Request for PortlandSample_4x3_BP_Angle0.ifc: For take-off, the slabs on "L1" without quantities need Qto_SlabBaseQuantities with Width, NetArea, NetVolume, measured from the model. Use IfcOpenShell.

First a look at what the model holds.

```python
import ifcopenshell
import ifcopenshell.util.element
import ifcopenshell.util.unit

model = ifcopenshell.open("PortlandSample_4x3_BP_Angle0.ifc")
print(model.schema)
for unit_type in ("LENGTHUNIT", "AREAUNIT", "VOLUMEUNIT"):
    print(unit_type, ifcopenshell.util.unit.calculate_unit_scale(model, unit_type))
storey = next(s for s in model.by_type("IfcBuildingStorey") if s.Name == "L1")
slabs = [e for e in ifcopenshell.util.element.get_decomposition(storey) if e.is_a("IfcSlab")]
for e in sorted(slabs, key=lambda e: e.id()):
    print(e.id(), e.is_a(), e.Name, list(ifcopenshell.util.element.get_psets(e, qtos_only=True)), sep=" | ")
```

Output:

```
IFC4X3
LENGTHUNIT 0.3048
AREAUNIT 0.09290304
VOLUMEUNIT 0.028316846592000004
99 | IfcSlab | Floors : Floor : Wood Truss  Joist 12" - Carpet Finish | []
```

```python
import ifcopenshell
import ifcopenshell.api.pset
import ifcopenshell.geom
import ifcopenshell.util.element
import ifcopenshell.util.shape
import ifcopenshell.util.unit

model = ifcopenshell.open("PortlandSample_4x3_BP_Angle0.ifc")
unit_scale = ifcopenshell.util.unit.calculate_unit_scale(model)
area_scale = ifcopenshell.util.unit.calculate_unit_scale(model, "AREAUNIT")
volume_scale = ifcopenshell.util.unit.calculate_unit_scale(model, "VOLUMEUNIT")
settings = ifcopenshell.geom.settings()

storey = next(s for s in model.by_type("IfcBuildingStorey") if s.Name == "L1")
slabs = [e for e in ifcopenshell.util.element.get_decomposition(storey) if e.is_a("IfcSlab")]

for e in sorted(slabs, key=lambda e: e.id()):
    if ifcopenshell.util.element.get_psets(e, qtos_only=True, should_inherit=False):
        continue
    # Geometry comes back in metres, in the element's own axes.
    shape = ifcopenshell.geom.create_shape(settings, e)
    values = {
        "Width": ifcopenshell.util.shape.get_z(shape.geometry) / unit_scale,
        "NetArea": ifcopenshell.util.shape.get_footprint_area(shape.geometry) / area_scale,
        "NetVolume": ifcopenshell.util.shape.get_volume(shape.geometry) / volume_scale,
    }
    qto = ifcopenshell.api.pset.add_qto(model, product=e, name="Qto_SlabBaseQuantities")
    ifcopenshell.api.pset.edit_qto(model, qto=qto, properties=values)
    print(e.id(), {k: round(v, 3) for k, v in values.items()})

model.write("PortlandSample_4x3_BP_Angle0_updated.ifc")
```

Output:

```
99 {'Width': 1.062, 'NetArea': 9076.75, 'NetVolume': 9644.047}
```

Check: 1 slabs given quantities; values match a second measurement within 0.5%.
